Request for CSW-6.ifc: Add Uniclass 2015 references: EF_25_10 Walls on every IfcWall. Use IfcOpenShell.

First a look at what the model holds.

```python
import ifcopenshell

model = ifcopenshell.open("CSW-6.ifc")
print(model.schema)
print("classifications:", [c.Name for c in model.by_type("IfcClassification")])
for ifc_class in ("IfcDoor", "IfcRoof", "IfcStair", "IfcWall", "IfcWindow"):
    print(ifc_class, len(model.by_type(ifc_class)))
```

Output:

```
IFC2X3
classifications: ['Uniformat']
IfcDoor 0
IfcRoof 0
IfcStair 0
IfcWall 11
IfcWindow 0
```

```python
import ifcopenshell
import ifcopenshell.api.classification

model = ifcopenshell.open("CSW-6.ifc")

# IFC2X3 requires Source and Edition and has no link from the project to the system.
system = model.create_entity("IfcClassification", Source="NBS", Edition="2015", Name="Uniclass 2015")

codes = {
    "IfcWall": ("EF_25_10", "Walls"),
}
for ifc_class, (code, name) in codes.items():
    products = model.by_type(ifc_class)
    ifcopenshell.api.classification.add_reference(
        model, products=products, classification=system, identification=code, name=name
    )
    print(code, len(products))

model.write("CSW-6-out.ifc")
```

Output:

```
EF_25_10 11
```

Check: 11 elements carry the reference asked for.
